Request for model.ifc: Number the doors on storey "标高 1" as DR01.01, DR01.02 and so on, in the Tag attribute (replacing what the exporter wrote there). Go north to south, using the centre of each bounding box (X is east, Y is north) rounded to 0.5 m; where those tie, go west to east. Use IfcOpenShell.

First a look at what the model holds.

```python
import ifcopenshell
import ifcopenshell.util.element
import ifcopenshell.util.placement

model = ifcopenshell.open("model.ifc")
print(model.schema)
storey = next(s for s in model.by_type("IfcBuildingStorey") if s.Name == "标高 1")
doors = [e for e in ifcopenshell.util.element.get_decomposition(storey) if e.is_a("IfcDoor")]
for e in sorted(doors, key=lambda e: e.id()):
    origin = ifcopenshell.util.placement.get_local_placement(e.ObjectPlacement)[:3, 3]
    print(e.id(), e.Tag, e.Name, origin.round(2) + 0.0, sep=" | ")
```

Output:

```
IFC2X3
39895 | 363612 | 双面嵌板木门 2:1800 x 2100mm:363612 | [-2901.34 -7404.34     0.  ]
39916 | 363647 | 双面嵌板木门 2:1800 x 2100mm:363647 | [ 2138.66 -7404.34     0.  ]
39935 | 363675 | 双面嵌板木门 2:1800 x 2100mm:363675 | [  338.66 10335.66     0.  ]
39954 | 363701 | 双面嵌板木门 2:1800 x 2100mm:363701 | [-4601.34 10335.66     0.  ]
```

```python
import ifcopenshell
import ifcopenshell.geom
import ifcopenshell.util.element
import ifcopenshell.util.shape

model = ifcopenshell.open("model.ifc")
settings = ifcopenshell.geom.settings()
settings.set("use-world-coords", True)


def centre(element):
    shape = ifcopenshell.geom.create_shape(settings, element)
    return ifcopenshell.util.shape.get_bbox_centroid(shape.geometry)


storey = next(s for s in model.by_type("IfcBuildingStorey") if s.Name == "标高 1")
doors = [e for e in ifcopenshell.util.element.get_decomposition(storey) if e.is_a("IfcDoor")]

# Insertion points can sit at a corner or the storey origin, so sort by the geometry (in metres).
centres = {e: centre(e) for e in doors}
doors.sort(key=lambda e: (-round(centres[e][1] / 0.5), centres[e][0]))

for i, e in enumerate(doors, start=1):
    number = f"DR01.{i:02d}"
    e.Tag = number
    print(e.id(), number)

model.write("model_updated.ifc")
```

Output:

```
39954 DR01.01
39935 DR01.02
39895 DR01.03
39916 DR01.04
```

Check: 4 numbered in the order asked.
